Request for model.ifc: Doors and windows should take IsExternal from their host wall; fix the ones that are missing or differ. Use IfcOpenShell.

First a look at what the model holds.

```python
import ifcopenshell
import ifcopenshell.util.element

model = ifcopenshell.open("model.ifc")
print(model.schema)
seen = {}
for e in model.by_type("IfcDoor") + model.by_type("IfcWindow"):
    if not e.FillsVoids:
        continue
    host = e.FillsVoids[0].RelatingOpeningElement.VoidsElements[0].RelatingBuildingElement
    own = ifcopenshell.util.element.get_pset(e, f"Pset_{e.is_a()[3:].removesuffix('StandardCase')}Common", "IsExternal")
    wall = ifcopenshell.util.element.get_pset(host, "Pset_WallCommon", "IsExternal")
    seen[e.is_a(), own, wall] = seen.get((e.is_a(), own, wall), 0) + 1
for (cls, own, wall), count in sorted(seen.items(), key=str):
    print(count, cls, "IsExternal:", own, "| host wall:", wall)
```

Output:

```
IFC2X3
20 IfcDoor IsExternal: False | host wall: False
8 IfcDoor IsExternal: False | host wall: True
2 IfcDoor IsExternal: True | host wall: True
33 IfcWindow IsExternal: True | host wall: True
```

```python
import ifcopenshell
import ifcopenshell.api.pset
import ifcopenshell.util.element

model = ifcopenshell.open("model.ifc")

count = 0
for ifc_class, pset_name in (("IfcDoor", "Pset_DoorCommon"), ("IfcWindow", "Pset_WindowCommon")):
    for e in model.by_type(ifc_class):
        if not e.FillsVoids:
            continue
        host = e.FillsVoids[0].RelatingOpeningElement.VoidsElements[0].RelatingBuildingElement
        external = ifcopenshell.util.element.get_pset(host, "Pset_WallCommon", "IsExternal")
        if external is None or ifcopenshell.util.element.get_pset(e, pset_name, "IsExternal") == external:
            continue
        pset = ifcopenshell.api.pset.add_pset(model, product=e, name=pset_name)
        ifcopenshell.api.pset.edit_pset(model, pset=pset, properties={"IsExternal": external})
        count += 1

print(count, "updated")

model.write("model_v2.ifc")
```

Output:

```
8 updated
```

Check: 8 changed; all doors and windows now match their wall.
